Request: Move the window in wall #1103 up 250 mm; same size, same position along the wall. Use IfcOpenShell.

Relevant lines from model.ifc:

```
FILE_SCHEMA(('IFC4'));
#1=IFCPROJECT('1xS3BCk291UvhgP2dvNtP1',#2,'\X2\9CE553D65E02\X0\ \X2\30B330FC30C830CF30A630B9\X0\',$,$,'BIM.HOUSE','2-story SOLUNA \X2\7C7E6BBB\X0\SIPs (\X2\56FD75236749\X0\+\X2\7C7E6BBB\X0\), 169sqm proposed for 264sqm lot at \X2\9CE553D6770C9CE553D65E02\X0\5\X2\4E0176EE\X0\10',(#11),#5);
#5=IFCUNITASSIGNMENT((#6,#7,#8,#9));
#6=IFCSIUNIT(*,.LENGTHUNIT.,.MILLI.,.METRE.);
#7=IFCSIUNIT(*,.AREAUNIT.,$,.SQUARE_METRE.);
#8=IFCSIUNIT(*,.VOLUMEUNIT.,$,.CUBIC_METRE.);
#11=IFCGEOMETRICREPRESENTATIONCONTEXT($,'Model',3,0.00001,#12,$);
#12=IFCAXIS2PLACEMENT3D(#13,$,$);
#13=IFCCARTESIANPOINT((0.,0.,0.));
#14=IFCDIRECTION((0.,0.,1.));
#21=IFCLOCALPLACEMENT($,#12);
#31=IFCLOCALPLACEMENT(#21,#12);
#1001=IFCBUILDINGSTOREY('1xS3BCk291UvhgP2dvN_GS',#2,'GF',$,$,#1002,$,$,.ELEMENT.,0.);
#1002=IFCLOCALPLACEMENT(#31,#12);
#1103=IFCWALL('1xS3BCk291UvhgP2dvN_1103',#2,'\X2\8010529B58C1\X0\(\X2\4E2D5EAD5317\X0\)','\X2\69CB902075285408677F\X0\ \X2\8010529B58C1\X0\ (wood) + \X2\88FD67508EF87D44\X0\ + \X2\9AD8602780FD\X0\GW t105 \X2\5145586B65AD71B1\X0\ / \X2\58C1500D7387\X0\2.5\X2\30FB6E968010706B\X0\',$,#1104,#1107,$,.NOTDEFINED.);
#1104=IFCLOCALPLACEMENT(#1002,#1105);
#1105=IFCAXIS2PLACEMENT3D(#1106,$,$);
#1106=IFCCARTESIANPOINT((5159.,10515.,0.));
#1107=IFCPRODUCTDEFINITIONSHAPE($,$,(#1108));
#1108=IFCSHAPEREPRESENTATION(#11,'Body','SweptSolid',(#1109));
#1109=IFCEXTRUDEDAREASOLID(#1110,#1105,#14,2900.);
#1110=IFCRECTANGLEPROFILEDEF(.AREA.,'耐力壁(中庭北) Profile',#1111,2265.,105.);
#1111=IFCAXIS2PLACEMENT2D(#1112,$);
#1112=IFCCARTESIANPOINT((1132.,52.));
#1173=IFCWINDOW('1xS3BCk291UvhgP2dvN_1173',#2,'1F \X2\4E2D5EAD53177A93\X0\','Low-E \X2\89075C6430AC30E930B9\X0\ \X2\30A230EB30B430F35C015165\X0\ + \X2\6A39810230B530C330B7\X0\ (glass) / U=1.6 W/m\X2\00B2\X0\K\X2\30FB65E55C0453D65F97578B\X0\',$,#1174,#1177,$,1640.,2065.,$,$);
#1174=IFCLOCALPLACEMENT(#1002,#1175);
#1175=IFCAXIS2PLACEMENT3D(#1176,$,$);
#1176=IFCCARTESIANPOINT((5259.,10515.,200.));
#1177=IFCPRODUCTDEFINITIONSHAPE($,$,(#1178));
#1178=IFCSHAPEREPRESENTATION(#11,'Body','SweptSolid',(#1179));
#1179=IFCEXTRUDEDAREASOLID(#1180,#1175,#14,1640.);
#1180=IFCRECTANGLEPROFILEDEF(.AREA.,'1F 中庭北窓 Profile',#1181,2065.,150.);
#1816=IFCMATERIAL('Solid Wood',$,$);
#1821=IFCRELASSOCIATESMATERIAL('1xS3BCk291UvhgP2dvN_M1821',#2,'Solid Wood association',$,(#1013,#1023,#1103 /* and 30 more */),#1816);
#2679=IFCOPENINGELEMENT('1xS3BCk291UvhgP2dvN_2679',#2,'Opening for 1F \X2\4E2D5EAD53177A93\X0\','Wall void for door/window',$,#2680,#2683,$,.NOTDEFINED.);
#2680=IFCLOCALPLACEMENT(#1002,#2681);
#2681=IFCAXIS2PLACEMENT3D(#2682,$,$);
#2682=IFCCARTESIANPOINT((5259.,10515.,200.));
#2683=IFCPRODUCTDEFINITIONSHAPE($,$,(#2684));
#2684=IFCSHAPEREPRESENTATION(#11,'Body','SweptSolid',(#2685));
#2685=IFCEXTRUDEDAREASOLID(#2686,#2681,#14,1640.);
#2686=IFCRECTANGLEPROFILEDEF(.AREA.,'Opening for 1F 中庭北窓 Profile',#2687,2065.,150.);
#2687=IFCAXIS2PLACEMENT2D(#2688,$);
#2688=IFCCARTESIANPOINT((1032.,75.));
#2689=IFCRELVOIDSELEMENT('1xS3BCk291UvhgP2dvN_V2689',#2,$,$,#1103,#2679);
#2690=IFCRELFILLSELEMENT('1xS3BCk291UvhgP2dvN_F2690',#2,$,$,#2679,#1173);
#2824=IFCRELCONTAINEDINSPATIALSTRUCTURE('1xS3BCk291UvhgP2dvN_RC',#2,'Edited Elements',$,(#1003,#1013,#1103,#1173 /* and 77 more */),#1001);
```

```python
import numpy as np
import ifcopenshell
import ifcopenshell.api.geometry
import ifcopenshell.util.placement
import ifcopenshell.util.unit

model = ifcopenshell.open("model.ifc")
unit_scale = ifcopenshell.util.unit.calculate_unit_scale(model)

window = model.by_guid("1xS3BCk291UvhgP2dvN_1173")
opening = window.FillsVoids[0].RelatingOpeningElement
dz = 0.25 / unit_scale

shift = np.array([0.0, 0.0, dz])
# The window is not placed relative to its opening, so move both.
for product in (opening, window):
    matrix = ifcopenshell.util.placement.get_local_placement(product.ObjectPlacement)
    matrix[:3, 3] += shift
    ifcopenshell.api.geometry.edit_object_placement(model, product=product, matrix=matrix, is_si=False)

print(f"moved by {dz * unit_scale:+.3f} m")

model.write("model-out.ifc")
```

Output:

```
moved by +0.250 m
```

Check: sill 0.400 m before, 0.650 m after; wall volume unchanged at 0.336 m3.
